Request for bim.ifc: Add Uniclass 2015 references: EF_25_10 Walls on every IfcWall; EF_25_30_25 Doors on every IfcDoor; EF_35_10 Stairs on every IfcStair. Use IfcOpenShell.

First a look at what the model holds.

```python
import ifcopenshell

model = ifcopenshell.open("bim.ifc")
print(model.schema)
print("classifications:", [c.Name for c in model.by_type("IfcClassification")])
for ifc_class in ("IfcDoor", "IfcRoof", "IfcStair", "IfcWall", "IfcWindow"):
    print(ifc_class, len(model.by_type(ifc_class)))
```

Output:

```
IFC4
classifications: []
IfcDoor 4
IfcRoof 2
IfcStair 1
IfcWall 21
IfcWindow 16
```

```python
import ifcopenshell
import ifcopenshell.api.classification

model = ifcopenshell.open("bim.ifc")

system = ifcopenshell.api.classification.add_classification(model, classification="Uniclass 2015")

codes = {
    "IfcWall": ("EF_25_10", "Walls"),
    "IfcDoor": ("EF_25_30_25", "Doors"),
    "IfcStair": ("EF_35_10", "Stairs"),
}
for ifc_class, (code, name) in codes.items():
    products = model.by_type(ifc_class)
    ifcopenshell.api.classification.add_reference(
        model, products=products, classification=system, identification=code, name=name
    )
    print(code, len(products))

model.write("bim-out.ifc")
```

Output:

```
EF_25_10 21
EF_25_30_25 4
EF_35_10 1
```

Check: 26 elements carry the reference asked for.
